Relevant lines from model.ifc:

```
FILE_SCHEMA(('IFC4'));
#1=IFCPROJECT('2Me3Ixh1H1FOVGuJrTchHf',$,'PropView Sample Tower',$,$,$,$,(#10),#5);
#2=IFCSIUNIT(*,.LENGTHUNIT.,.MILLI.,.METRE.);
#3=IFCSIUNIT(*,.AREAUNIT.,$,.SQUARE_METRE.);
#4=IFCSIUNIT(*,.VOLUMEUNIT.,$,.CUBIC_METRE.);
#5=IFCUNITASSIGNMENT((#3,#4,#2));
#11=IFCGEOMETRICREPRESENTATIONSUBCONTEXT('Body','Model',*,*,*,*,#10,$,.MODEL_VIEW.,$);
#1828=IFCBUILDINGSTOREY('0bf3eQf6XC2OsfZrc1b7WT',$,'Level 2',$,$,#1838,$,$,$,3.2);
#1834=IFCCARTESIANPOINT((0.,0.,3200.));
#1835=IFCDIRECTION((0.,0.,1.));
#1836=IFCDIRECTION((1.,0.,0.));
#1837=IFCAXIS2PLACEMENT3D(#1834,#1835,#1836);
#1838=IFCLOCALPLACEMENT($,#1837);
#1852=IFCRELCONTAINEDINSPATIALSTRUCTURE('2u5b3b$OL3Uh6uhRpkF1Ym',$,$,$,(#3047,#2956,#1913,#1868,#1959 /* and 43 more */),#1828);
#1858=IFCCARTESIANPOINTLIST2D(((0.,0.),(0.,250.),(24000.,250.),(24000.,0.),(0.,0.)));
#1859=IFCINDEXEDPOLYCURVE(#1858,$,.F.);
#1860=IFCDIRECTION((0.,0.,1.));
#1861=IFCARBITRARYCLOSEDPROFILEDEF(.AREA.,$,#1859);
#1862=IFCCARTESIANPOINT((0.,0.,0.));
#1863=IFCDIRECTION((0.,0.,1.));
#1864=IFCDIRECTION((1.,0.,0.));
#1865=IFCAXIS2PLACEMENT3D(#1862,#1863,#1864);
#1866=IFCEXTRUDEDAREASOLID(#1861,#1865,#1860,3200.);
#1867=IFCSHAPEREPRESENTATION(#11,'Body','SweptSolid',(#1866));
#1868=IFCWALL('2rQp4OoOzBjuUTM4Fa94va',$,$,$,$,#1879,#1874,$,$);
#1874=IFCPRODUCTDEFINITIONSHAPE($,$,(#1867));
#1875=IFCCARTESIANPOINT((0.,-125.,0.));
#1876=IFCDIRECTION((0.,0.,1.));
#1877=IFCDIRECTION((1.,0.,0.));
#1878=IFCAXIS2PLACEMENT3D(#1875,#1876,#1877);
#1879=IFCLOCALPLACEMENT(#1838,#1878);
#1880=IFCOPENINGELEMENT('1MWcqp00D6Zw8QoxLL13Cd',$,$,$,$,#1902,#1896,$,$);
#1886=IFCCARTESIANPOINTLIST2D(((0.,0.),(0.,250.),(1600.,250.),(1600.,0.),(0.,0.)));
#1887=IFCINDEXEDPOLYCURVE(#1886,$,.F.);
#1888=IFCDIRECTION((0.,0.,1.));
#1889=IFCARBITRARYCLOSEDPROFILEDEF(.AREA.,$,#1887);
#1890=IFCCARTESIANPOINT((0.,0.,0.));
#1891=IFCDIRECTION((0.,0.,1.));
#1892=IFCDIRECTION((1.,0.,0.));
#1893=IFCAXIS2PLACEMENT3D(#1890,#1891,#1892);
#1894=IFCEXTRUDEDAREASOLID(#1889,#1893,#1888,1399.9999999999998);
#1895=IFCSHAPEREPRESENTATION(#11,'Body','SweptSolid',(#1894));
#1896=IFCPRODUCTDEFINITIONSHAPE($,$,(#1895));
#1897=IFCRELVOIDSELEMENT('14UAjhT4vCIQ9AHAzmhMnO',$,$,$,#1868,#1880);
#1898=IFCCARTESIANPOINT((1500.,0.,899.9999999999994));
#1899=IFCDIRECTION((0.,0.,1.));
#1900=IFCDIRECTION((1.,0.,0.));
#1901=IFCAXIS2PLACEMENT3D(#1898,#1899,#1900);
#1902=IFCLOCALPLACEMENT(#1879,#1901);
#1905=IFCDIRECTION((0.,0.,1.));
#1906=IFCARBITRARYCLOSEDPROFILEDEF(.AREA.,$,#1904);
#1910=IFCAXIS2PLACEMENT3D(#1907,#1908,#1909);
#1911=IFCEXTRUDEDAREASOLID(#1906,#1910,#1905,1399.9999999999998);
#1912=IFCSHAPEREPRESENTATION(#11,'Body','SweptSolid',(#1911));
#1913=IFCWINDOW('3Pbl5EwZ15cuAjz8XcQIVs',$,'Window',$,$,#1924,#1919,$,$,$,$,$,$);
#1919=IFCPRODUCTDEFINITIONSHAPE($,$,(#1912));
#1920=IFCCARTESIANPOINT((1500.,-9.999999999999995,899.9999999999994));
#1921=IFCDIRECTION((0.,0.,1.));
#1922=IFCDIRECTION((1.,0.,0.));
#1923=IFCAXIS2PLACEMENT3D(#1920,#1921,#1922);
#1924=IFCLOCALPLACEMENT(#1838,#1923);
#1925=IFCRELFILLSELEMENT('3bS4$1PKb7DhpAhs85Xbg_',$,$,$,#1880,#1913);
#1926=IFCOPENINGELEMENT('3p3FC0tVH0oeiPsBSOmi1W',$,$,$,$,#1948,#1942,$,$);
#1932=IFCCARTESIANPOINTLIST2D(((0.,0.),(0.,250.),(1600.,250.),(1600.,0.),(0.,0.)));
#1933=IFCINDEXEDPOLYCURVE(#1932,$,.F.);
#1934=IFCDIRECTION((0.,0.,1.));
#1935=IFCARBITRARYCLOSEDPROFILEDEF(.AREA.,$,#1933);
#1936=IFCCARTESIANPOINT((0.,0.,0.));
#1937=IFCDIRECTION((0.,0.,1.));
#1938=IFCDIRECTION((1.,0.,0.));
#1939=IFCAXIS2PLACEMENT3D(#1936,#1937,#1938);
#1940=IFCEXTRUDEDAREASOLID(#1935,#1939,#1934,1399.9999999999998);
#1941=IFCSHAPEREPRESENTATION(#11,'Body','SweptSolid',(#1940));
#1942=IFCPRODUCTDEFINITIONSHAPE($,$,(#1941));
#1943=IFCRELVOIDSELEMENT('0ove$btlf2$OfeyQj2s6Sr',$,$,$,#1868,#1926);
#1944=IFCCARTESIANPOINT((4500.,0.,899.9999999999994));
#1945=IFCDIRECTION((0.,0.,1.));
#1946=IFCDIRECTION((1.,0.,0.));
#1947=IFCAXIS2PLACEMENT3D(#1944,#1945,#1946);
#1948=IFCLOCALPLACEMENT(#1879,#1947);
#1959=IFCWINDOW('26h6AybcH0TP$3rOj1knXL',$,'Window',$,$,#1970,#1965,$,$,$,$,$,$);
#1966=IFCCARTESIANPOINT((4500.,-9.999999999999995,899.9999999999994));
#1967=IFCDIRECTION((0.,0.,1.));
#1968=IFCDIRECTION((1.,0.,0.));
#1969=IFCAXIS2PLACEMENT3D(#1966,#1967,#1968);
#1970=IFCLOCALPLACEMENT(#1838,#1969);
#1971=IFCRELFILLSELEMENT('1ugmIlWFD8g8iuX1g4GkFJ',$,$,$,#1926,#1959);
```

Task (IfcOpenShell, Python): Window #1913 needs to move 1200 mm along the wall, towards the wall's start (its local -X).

```python
import ifcopenshell
import ifcopenshell.api.geometry
import ifcopenshell.util.placement

model = ifcopenshell.open("model.ifc")

window = model.by_guid("3Pbl5EwZ15cuAjz8XcQIVs")
opening = window.FillsVoids[0].RelatingOpeningElement
wall = opening.VoidsElements[0].RelatingBuildingElement

wall_matrix = ifcopenshell.util.placement.get_local_placement(wall.ObjectPlacement)
shift = wall_matrix[:3, 0] * -1200.0
before = ifcopenshell.util.placement.get_local_placement(window.ObjectPlacement)[:3, 3].copy()

# The window is not placed relative to its opening, so move both.
for product in (opening, window):
    matrix = ifcopenshell.util.placement.get_local_placement(product.ObjectPlacement)
    matrix[:3, 3] += shift
    ifcopenshell.api.geometry.edit_object_placement(model, product=product, matrix=matrix, is_si=False)

after = ifcopenshell.util.placement.get_local_placement(window.ObjectPlacement)[:3, 3]
print("window moved by", (after - before).round(3) + 0.0)

model.write("model_v2.ifc")
```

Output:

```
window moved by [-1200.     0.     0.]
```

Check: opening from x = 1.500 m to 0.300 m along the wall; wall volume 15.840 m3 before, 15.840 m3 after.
